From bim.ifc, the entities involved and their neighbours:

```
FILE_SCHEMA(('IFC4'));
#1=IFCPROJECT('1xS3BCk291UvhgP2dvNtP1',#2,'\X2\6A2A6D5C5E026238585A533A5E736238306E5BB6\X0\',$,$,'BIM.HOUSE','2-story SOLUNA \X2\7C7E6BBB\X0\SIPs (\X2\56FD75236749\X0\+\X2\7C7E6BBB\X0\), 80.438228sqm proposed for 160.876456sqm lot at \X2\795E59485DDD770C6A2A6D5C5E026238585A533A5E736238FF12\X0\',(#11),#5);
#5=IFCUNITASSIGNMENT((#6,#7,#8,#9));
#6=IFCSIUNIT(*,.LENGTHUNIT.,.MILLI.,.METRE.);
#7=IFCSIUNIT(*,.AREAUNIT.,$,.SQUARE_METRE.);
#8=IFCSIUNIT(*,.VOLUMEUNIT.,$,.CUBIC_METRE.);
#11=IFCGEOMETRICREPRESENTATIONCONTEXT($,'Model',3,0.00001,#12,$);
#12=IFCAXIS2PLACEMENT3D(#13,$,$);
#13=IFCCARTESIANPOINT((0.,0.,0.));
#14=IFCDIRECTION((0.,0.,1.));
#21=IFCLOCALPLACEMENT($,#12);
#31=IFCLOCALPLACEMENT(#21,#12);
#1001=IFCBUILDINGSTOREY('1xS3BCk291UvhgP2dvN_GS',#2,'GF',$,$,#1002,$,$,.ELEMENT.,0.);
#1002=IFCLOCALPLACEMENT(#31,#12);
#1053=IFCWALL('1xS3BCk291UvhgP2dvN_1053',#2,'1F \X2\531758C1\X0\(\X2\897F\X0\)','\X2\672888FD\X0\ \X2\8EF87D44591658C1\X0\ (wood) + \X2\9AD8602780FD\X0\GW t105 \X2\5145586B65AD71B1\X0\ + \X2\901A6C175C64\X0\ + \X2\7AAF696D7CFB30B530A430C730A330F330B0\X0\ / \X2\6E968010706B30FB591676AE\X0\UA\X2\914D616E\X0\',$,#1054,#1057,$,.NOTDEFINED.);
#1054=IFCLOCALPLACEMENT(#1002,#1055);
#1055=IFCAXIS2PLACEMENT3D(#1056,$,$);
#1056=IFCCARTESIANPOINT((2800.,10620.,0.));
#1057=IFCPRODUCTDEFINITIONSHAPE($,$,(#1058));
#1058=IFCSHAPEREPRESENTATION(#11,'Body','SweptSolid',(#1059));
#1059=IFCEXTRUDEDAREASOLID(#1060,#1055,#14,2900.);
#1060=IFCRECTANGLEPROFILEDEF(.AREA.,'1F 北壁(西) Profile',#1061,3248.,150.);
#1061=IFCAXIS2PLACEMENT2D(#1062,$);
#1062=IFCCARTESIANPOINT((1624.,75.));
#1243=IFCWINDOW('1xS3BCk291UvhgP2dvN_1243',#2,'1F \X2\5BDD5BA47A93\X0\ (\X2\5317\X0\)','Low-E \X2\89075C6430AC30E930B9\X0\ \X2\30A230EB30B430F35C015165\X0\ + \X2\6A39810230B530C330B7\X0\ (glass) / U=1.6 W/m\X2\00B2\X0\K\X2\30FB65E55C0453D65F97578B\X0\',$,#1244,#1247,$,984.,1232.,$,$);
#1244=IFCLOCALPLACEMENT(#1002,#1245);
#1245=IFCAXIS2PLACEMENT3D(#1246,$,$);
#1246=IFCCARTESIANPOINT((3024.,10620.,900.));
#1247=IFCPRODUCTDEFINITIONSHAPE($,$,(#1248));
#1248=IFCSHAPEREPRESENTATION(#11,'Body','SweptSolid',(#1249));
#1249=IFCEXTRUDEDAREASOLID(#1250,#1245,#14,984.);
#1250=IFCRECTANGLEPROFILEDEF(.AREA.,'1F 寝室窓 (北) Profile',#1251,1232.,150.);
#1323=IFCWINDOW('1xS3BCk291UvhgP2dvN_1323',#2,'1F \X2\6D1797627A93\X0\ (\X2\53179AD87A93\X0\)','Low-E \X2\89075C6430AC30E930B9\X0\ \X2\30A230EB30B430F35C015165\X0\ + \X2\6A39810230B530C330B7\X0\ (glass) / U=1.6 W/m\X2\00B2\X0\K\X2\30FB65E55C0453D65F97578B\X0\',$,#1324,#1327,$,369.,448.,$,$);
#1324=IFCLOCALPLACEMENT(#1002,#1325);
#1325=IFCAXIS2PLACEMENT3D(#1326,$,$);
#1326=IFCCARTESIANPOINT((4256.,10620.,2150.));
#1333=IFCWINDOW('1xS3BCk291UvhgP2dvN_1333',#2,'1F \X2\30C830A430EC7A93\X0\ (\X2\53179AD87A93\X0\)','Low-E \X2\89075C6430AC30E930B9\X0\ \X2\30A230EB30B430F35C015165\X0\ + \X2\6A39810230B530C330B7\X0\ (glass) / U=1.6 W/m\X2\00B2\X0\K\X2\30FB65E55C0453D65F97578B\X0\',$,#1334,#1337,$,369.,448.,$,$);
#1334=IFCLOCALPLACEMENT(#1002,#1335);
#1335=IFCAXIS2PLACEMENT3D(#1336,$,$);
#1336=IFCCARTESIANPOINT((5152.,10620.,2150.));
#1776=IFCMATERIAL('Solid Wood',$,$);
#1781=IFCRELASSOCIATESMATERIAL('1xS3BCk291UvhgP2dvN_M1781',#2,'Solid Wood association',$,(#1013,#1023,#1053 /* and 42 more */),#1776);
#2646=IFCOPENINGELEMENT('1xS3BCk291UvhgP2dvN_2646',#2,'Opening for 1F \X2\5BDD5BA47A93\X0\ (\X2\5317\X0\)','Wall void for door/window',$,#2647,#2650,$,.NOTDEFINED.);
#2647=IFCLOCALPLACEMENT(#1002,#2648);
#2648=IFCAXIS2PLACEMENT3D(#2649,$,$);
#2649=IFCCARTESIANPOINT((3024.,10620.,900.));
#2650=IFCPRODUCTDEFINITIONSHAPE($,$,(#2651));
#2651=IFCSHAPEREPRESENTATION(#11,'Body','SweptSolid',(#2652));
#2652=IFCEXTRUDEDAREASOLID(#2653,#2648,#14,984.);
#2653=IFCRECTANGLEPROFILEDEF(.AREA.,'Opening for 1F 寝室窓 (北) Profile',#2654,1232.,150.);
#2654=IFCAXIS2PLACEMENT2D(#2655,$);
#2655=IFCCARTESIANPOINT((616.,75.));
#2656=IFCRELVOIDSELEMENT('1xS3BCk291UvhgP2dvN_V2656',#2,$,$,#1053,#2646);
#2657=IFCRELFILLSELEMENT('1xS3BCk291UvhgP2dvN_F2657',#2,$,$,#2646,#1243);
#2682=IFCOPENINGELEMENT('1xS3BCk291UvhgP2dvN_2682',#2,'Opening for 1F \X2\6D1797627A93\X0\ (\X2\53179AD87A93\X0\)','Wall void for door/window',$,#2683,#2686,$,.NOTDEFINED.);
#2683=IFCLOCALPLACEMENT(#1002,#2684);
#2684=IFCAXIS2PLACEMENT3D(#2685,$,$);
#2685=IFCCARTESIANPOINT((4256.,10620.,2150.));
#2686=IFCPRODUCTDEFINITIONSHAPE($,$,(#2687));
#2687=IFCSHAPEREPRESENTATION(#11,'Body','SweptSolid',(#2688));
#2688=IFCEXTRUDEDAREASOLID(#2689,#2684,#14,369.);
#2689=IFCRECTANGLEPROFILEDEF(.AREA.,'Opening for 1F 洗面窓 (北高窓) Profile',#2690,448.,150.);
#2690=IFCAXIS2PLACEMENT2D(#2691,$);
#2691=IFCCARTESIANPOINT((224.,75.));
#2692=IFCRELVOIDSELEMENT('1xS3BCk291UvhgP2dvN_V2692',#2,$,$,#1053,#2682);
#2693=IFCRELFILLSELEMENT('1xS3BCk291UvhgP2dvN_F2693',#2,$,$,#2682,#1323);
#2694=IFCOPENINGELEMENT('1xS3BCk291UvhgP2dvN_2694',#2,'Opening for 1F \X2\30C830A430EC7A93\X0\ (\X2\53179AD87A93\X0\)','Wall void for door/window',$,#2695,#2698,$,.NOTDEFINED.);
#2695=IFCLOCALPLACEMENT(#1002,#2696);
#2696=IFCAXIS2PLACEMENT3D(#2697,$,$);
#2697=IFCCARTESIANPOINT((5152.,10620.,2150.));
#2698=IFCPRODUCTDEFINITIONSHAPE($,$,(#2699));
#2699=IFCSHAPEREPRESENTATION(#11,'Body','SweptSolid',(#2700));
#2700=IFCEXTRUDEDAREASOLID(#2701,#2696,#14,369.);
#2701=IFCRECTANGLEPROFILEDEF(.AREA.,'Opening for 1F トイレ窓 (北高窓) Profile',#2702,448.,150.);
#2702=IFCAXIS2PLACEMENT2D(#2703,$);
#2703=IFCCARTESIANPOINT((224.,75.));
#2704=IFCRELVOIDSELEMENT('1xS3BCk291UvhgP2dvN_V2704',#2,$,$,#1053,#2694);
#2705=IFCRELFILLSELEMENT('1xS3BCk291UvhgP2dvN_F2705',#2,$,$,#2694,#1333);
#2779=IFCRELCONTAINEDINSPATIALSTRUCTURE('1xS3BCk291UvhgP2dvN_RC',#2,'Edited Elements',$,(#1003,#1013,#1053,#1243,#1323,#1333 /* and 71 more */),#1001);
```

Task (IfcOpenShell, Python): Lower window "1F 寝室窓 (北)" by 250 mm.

```python
import numpy as np
import ifcopenshell
import ifcopenshell.api.geometry
import ifcopenshell.util.placement
import ifcopenshell.util.unit

model = ifcopenshell.open("bim.ifc")
unit_scale = ifcopenshell.util.unit.calculate_unit_scale(model)

window = model.by_guid("1xS3BCk291UvhgP2dvN_1243")
opening = window.FillsVoids[0].RelatingOpeningElement
dz = -250.0

shift = np.array([0.0, 0.0, dz])
# The window is not placed relative to its opening, so move both.
for product in (opening, window):
    matrix = ifcopenshell.util.placement.get_local_placement(product.ObjectPlacement)
    matrix[:3, 3] += shift
    ifcopenshell.api.geometry.edit_object_placement(model, product=product, matrix=matrix, is_si=False)

print(f"moved by {dz * unit_scale:+.3f} m")

model.write("bim_rev.ifc")
```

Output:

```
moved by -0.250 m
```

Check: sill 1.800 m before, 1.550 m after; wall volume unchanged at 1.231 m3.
